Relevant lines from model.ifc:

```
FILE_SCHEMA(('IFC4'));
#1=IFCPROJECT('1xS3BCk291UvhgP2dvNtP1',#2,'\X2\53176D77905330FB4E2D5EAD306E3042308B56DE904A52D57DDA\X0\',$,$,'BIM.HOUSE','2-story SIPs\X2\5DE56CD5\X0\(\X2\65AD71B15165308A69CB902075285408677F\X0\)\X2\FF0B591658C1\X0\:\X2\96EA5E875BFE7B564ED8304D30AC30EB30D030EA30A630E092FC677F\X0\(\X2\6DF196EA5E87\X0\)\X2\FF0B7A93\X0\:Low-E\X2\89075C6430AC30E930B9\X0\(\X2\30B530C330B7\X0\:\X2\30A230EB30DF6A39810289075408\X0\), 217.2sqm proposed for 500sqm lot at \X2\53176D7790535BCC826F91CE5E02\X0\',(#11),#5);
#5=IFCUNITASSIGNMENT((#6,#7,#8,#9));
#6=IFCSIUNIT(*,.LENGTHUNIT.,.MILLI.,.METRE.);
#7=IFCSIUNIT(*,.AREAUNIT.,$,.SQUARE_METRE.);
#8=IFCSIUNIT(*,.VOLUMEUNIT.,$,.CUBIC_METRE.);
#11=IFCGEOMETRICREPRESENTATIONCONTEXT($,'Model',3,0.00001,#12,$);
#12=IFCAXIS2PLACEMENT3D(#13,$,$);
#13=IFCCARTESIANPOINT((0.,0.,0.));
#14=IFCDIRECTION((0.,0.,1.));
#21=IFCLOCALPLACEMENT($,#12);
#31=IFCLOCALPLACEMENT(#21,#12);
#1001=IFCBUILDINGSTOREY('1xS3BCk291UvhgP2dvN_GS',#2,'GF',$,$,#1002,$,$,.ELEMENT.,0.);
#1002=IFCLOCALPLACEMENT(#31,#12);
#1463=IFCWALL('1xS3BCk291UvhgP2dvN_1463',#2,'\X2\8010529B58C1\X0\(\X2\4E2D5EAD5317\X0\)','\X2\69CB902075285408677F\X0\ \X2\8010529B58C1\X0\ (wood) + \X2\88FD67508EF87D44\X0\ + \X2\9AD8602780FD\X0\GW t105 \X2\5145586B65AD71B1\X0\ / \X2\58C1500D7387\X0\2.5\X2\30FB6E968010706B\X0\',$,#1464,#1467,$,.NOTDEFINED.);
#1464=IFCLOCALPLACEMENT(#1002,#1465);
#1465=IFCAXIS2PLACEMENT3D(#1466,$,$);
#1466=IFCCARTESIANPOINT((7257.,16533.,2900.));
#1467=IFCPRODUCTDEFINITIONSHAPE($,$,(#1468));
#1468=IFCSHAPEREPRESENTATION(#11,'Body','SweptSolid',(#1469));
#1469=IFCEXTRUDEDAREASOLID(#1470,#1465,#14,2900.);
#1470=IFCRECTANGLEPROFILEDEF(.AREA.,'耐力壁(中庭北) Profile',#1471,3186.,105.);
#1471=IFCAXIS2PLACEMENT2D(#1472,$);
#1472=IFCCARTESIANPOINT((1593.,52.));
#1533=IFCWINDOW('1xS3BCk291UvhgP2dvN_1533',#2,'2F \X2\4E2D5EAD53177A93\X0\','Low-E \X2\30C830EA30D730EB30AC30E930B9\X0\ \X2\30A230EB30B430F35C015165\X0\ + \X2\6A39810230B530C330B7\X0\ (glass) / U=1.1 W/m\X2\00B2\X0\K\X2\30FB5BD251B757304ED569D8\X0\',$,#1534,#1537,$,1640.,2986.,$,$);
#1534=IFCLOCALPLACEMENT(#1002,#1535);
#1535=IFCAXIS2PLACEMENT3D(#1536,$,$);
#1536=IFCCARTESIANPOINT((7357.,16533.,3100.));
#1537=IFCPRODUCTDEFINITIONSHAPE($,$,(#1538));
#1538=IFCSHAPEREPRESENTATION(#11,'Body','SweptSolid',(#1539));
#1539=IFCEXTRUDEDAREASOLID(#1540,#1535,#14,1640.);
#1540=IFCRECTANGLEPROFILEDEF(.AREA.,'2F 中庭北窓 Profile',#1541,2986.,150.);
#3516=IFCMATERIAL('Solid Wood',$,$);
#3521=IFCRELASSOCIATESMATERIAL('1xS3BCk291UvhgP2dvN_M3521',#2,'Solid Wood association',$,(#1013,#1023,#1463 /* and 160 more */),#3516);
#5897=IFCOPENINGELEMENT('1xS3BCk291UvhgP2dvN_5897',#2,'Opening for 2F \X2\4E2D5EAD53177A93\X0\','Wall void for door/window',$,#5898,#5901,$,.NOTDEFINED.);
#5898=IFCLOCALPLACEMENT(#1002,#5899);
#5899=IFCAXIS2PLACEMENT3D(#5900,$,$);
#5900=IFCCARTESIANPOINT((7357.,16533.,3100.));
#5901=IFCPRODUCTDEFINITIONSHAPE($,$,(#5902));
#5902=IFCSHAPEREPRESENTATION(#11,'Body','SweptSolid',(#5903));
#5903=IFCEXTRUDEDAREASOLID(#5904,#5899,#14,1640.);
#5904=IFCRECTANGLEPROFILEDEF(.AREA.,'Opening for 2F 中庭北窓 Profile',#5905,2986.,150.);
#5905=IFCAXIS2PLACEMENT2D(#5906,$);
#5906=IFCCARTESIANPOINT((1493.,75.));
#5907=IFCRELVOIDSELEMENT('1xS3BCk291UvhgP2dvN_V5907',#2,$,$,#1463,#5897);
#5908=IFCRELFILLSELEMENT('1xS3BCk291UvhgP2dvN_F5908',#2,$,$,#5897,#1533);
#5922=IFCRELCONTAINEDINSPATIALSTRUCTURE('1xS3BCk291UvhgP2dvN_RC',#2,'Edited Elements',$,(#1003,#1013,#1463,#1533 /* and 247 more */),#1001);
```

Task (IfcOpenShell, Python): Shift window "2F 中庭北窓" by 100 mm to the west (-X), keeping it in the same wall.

```python
import ifcopenshell
import ifcopenshell.api.geometry
import ifcopenshell.util.placement
import ifcopenshell.util.unit

model = ifcopenshell.open("model.ifc")
unit_scale = ifcopenshell.util.unit.calculate_unit_scale(model)

window = model.by_guid("1xS3BCk291UvhgP2dvN_1533")
opening = window.FillsVoids[0].RelatingOpeningElement
wall = opening.VoidsElements[0].RelatingBuildingElement

wall_matrix = ifcopenshell.util.placement.get_local_placement(wall.ObjectPlacement)
shift = wall_matrix[:3, 0] * -0.1 / unit_scale
before = ifcopenshell.util.placement.get_local_placement(window.ObjectPlacement)[:3, 3].copy()

# The window is not placed relative to its opening, so move both.
for product in (opening, window):
    matrix = ifcopenshell.util.placement.get_local_placement(product.ObjectPlacement)
    matrix[:3, 3] += shift
    ifcopenshell.api.geometry.edit_object_placement(model, product=product, matrix=matrix, is_si=False)

after = ifcopenshell.util.placement.get_local_placement(window.ObjectPlacement)[:3, 3]
print("window moved by", (after - before).round(3) + 0.0)

model.write("model_updated.ifc")
```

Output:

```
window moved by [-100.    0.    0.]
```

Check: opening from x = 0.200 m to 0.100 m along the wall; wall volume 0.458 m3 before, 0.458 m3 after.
